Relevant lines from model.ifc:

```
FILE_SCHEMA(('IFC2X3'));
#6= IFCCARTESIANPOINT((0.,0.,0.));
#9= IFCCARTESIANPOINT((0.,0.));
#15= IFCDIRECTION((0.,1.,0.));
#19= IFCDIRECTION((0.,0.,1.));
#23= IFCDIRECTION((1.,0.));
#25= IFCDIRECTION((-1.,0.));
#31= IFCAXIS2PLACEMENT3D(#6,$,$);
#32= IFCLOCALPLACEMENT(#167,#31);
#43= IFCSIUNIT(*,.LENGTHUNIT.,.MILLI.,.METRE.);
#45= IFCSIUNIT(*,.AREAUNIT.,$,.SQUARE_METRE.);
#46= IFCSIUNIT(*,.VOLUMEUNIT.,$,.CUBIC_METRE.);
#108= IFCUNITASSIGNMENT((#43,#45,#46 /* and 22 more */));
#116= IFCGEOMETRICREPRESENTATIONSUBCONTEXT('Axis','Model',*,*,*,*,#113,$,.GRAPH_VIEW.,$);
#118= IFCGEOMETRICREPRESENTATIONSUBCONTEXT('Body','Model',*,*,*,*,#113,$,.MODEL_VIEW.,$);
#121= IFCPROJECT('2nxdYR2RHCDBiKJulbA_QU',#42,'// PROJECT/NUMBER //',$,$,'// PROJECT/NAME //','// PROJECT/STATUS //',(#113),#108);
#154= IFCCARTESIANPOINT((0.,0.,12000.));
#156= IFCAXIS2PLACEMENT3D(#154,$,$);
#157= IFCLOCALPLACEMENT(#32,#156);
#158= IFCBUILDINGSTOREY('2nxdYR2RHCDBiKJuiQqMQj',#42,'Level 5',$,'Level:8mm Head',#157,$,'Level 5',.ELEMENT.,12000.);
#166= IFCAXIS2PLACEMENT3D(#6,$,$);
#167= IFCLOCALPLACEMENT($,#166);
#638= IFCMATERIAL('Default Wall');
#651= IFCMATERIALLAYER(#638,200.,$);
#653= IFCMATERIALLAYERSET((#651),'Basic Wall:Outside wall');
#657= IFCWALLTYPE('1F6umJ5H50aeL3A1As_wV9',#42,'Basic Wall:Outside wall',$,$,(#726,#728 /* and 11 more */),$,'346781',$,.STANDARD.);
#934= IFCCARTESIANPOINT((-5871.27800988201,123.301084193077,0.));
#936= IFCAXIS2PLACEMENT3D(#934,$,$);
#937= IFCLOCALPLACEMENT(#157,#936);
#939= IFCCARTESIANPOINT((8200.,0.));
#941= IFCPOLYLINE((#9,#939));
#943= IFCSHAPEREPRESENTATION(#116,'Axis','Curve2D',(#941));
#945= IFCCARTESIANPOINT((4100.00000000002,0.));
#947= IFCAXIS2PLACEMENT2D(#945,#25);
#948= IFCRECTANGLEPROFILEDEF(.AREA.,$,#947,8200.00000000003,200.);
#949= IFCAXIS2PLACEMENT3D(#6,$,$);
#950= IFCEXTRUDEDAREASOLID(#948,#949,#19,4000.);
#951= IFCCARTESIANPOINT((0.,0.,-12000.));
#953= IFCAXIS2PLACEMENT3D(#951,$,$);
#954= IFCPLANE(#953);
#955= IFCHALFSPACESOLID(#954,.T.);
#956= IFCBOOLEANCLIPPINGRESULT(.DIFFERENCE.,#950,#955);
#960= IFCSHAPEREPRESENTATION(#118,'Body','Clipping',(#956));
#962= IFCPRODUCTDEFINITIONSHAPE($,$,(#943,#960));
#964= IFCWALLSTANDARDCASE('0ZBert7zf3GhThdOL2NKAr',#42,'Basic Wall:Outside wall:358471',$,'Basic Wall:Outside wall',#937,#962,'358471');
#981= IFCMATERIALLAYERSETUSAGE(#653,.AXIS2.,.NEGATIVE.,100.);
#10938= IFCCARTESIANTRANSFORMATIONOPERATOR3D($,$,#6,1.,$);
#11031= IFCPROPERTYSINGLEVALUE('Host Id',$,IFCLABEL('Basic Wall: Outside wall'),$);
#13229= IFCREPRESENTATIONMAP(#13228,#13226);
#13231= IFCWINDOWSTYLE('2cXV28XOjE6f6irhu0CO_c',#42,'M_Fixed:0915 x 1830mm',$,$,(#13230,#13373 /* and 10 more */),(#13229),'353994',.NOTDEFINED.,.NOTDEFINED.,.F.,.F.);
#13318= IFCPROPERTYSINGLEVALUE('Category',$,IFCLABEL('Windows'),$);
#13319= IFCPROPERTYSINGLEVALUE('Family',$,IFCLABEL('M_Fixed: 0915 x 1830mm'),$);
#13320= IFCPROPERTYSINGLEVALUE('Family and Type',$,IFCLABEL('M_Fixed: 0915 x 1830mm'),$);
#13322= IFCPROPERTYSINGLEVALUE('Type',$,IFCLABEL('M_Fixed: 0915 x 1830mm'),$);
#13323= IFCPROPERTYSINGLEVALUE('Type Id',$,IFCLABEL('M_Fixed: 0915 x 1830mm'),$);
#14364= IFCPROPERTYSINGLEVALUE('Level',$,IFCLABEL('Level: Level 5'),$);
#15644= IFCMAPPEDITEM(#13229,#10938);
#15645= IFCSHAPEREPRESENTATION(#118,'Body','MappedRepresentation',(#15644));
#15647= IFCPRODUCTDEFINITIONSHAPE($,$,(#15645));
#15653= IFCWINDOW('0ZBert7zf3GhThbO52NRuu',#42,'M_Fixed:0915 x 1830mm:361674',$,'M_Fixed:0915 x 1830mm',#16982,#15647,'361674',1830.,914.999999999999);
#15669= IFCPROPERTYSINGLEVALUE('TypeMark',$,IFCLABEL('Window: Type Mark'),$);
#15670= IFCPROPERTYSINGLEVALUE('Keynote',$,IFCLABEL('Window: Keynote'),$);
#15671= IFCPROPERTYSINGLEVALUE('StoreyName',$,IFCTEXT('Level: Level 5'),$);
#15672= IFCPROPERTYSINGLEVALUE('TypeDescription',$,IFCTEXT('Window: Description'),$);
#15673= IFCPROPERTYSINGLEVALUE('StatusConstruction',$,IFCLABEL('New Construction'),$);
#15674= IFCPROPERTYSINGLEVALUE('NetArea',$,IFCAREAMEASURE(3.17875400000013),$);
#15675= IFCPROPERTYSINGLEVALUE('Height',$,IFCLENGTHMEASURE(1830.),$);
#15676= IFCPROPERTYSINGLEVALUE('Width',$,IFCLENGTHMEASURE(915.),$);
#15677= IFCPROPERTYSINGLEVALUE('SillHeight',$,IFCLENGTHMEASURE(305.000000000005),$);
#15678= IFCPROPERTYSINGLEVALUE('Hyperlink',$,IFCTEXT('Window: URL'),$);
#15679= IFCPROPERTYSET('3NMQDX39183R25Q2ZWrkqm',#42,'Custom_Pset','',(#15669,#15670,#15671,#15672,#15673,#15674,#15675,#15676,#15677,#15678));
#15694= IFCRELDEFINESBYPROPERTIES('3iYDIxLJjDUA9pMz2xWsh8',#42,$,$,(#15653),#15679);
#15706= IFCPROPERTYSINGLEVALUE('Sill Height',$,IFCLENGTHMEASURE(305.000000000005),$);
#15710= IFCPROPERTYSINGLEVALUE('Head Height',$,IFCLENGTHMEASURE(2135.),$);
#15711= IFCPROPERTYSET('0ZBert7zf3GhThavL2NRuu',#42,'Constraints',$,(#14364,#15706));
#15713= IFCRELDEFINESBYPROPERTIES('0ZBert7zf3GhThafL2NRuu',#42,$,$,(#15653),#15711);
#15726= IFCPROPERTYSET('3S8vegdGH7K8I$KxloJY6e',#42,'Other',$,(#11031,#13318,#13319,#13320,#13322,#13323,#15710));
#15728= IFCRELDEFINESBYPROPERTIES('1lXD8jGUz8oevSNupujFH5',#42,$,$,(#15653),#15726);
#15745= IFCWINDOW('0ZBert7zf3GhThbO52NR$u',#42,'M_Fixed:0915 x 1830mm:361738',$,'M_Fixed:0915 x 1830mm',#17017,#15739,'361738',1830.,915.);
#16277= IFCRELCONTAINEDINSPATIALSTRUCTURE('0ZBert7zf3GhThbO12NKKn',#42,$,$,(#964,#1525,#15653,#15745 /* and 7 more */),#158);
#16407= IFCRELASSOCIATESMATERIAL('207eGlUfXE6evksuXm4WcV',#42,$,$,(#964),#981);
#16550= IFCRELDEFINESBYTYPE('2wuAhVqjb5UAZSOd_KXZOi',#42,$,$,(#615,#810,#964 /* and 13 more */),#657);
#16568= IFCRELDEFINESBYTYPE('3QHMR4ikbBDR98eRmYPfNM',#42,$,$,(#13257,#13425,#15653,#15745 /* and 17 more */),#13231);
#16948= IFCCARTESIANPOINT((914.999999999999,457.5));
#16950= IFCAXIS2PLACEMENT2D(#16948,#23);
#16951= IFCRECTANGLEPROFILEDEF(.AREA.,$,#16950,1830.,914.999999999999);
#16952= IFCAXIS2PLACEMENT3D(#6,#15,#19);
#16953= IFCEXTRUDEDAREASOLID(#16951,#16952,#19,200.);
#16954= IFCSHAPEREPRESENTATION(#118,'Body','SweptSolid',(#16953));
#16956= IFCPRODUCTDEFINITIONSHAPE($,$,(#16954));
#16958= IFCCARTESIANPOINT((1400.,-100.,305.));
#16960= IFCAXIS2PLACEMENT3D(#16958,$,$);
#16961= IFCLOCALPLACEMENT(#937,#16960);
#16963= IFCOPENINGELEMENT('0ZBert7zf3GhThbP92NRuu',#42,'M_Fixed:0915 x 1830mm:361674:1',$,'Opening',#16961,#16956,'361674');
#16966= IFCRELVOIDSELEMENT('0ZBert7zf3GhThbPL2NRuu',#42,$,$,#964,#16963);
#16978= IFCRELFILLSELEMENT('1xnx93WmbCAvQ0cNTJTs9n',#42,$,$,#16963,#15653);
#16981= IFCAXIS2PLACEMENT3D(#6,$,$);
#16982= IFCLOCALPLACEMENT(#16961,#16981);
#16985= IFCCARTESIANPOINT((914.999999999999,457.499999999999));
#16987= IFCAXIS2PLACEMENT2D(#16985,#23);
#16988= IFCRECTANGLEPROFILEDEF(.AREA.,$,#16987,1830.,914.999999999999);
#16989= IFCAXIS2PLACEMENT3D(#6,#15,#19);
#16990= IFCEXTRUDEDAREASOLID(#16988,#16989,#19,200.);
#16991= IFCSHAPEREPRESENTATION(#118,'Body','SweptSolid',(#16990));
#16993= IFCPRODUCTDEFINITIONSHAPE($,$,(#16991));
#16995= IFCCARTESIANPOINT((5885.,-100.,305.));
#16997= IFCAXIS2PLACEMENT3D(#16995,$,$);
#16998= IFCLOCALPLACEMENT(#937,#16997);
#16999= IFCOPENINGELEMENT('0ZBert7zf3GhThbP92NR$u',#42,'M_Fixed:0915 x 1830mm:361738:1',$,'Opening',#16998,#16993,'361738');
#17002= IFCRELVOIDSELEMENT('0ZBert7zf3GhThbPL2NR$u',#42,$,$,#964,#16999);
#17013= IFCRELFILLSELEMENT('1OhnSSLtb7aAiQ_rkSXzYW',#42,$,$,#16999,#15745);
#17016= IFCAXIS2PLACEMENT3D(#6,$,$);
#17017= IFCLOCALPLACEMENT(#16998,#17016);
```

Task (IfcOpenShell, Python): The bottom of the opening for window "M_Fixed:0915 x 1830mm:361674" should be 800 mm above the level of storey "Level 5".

```python
import numpy as np
import ifcopenshell
import ifcopenshell.api.geometry
import ifcopenshell.api.pset
import ifcopenshell.geom
import ifcopenshell.util.element
import ifcopenshell.util.placement
import ifcopenshell.util.shape
import ifcopenshell.util.unit

model = ifcopenshell.open("model.ifc")
unit_scale = ifcopenshell.util.unit.calculate_unit_scale(model)

window = model.by_guid("0ZBert7zf3GhThbO52NRuu")
opening = window.FillsVoids[0].RelatingOpeningElement
storey = ifcopenshell.util.element.get_container(window, ifc_class="IfcBuildingStorey")
level = ifcopenshell.util.placement.get_local_placement(storey.ObjectPlacement)[2, 3]

# The opening's origin need not be at the sill, so measure its lowest point.
shape = ifcopenshell.geom.create_shape(ifcopenshell.geom.settings(), opening)
bottom = ifcopenshell.util.shape.get_shape_bottom_elevation(shape, shape.geometry) / unit_scale
dz = level + 0.8 / unit_scale - bottom

shift = np.array([0.0, 0.0, dz])
# The window is placed relative to its opening, so it follows when the opening moves.
matrix = ifcopenshell.util.placement.get_local_placement(opening.ObjectPlacement)
matrix[:3, 3] += shift
ifcopenshell.api.geometry.edit_object_placement(
    model, product=opening, matrix=matrix, is_si=False, should_transform_children=True
)

# Keep the stored heights in step.
pset = model.by_id(ifcopenshell.util.element.get_pset(window, "Custom_Pset", should_inherit=False)["id"])
ifcopenshell.api.pset.edit_pset(model, pset=pset, properties={
    "SillHeight": model.create_entity("IfcLengthMeasure", ifcopenshell.util.element.get_pset(window, "Constraints", "Sill Height") + dz),
})
pset = model.by_id(ifcopenshell.util.element.get_pset(window, "Constraints", should_inherit=False)["id"])
ifcopenshell.api.pset.edit_pset(model, pset=pset, properties={
    "Sill Height": model.create_entity("IfcLengthMeasure", ifcopenshell.util.element.get_pset(window, "Constraints", "Sill Height") + dz),
})
pset = model.by_id(ifcopenshell.util.element.get_pset(window, "Other", should_inherit=False)["id"])
ifcopenshell.api.pset.edit_pset(model, pset=pset, properties={
    "Head Height": model.create_entity("IfcLengthMeasure", ifcopenshell.util.element.get_pset(window, "Other", "Head Height") + dz),
})

print(f"moved by {dz * unit_scale:+.3f} m")

model.write("model_edited.ifc")
```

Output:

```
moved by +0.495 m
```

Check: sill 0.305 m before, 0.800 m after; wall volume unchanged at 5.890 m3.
